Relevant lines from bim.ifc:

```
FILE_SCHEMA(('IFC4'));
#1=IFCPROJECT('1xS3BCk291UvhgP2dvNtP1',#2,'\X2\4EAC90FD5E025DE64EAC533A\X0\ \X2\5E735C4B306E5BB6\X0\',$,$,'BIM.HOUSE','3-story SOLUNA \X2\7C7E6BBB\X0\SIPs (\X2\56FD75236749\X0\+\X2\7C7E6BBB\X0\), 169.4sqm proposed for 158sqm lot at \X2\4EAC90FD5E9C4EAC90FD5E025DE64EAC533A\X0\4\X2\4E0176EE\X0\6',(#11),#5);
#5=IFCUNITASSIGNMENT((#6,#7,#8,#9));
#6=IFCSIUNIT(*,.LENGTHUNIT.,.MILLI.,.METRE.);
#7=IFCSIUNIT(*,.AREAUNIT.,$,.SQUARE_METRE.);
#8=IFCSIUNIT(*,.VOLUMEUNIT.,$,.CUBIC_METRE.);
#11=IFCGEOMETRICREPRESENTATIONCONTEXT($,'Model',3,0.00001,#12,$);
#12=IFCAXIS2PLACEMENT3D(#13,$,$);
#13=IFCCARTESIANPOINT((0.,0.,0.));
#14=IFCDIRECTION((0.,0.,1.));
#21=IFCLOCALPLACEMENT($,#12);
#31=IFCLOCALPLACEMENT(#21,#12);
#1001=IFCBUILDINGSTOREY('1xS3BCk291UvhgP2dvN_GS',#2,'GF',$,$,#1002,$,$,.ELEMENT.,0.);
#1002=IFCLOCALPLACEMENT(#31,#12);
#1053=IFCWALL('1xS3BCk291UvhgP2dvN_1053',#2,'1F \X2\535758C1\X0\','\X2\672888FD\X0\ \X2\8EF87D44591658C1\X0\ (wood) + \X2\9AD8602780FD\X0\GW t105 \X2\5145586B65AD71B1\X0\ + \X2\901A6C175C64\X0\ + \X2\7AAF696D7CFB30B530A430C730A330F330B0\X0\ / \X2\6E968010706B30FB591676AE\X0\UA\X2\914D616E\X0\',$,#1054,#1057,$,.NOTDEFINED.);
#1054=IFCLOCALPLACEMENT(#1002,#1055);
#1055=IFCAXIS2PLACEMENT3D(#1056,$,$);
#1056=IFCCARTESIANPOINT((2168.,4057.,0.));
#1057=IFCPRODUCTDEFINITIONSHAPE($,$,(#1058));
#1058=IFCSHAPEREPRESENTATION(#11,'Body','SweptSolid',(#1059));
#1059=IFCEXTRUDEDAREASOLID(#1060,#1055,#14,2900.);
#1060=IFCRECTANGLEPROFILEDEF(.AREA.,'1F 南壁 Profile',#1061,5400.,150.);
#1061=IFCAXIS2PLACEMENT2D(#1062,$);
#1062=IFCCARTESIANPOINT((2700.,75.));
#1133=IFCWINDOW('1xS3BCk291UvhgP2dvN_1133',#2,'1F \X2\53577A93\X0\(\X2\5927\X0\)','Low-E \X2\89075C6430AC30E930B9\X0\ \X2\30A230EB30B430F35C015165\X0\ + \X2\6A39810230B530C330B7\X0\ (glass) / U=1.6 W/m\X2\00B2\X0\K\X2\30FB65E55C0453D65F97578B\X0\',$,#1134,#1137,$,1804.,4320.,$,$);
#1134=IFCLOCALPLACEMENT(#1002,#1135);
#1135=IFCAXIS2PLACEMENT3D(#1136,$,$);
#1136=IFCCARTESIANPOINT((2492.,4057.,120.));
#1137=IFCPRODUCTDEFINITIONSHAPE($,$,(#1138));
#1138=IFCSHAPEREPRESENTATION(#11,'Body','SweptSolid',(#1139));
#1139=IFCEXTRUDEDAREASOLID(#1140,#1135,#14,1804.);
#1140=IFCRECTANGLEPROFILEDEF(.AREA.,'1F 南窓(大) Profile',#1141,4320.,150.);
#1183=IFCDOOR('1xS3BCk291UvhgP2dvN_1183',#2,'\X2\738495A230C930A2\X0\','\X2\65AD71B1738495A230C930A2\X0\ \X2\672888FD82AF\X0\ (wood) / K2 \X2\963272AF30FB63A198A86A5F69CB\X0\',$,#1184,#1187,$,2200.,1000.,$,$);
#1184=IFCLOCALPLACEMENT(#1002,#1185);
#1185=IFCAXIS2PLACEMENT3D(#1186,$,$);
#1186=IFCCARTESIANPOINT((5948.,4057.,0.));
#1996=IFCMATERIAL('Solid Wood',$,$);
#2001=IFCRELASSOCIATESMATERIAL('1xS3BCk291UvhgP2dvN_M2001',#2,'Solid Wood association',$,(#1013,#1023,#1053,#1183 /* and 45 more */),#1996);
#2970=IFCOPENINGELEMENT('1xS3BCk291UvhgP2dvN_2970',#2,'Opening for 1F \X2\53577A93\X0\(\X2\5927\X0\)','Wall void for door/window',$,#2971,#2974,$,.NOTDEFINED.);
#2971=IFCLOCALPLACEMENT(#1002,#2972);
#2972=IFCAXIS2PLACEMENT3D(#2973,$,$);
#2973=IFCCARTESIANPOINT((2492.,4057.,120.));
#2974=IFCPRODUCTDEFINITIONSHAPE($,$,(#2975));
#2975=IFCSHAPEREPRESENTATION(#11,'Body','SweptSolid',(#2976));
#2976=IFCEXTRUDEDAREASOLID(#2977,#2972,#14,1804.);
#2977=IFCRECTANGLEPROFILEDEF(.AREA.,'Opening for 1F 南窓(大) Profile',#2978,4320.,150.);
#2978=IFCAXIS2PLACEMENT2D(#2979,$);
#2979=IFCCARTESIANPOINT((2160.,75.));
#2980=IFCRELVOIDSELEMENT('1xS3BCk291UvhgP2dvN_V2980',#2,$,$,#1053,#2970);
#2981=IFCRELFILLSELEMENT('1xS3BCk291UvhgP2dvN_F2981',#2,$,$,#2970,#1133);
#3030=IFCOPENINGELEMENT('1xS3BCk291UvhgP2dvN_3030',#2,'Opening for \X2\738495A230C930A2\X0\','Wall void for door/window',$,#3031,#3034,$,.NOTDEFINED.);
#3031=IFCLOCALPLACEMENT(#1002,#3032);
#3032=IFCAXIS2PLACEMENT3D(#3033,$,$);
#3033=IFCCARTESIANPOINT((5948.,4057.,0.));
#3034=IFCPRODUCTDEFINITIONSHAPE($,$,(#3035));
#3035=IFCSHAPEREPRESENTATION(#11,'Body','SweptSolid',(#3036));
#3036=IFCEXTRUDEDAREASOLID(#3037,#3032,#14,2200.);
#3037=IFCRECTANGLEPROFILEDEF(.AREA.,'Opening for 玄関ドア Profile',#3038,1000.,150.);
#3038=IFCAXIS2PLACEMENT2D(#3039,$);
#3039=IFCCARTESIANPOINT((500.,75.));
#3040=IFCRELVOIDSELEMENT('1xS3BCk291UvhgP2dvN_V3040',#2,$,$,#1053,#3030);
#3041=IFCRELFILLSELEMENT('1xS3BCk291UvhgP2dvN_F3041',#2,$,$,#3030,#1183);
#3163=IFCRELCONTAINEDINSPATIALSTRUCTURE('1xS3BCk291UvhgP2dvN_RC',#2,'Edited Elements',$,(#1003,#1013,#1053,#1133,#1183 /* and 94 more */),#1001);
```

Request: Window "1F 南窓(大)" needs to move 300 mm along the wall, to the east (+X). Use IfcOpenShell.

```python
import ifcopenshell
import ifcopenshell.api.geometry
import ifcopenshell.util.placement

model = ifcopenshell.open("bim.ifc")

window = model.by_guid("1xS3BCk291UvhgP2dvN_1133")
opening = window.FillsVoids[0].RelatingOpeningElement
wall = opening.VoidsElements[0].RelatingBuildingElement

wall_matrix = ifcopenshell.util.placement.get_local_placement(wall.ObjectPlacement)
shift = wall_matrix[:3, 0] * 300.0
before = ifcopenshell.util.placement.get_local_placement(window.ObjectPlacement)[:3, 3].copy()

# The window is not placed relative to its opening, so move both.
for product in (opening, window):
    matrix = ifcopenshell.util.placement.get_local_placement(product.ObjectPlacement)
    matrix[:3, 3] += shift
    ifcopenshell.api.geometry.edit_object_placement(model, product=product, matrix=matrix, is_si=False)

after = ifcopenshell.util.placement.get_local_placement(window.ObjectPlacement)[:3, 3]
print("window moved by", (after - before).round(3) + 0.0)

model.write("bim_updated.ifc")
```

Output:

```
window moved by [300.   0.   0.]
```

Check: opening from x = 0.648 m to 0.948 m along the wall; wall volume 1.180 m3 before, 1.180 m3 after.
